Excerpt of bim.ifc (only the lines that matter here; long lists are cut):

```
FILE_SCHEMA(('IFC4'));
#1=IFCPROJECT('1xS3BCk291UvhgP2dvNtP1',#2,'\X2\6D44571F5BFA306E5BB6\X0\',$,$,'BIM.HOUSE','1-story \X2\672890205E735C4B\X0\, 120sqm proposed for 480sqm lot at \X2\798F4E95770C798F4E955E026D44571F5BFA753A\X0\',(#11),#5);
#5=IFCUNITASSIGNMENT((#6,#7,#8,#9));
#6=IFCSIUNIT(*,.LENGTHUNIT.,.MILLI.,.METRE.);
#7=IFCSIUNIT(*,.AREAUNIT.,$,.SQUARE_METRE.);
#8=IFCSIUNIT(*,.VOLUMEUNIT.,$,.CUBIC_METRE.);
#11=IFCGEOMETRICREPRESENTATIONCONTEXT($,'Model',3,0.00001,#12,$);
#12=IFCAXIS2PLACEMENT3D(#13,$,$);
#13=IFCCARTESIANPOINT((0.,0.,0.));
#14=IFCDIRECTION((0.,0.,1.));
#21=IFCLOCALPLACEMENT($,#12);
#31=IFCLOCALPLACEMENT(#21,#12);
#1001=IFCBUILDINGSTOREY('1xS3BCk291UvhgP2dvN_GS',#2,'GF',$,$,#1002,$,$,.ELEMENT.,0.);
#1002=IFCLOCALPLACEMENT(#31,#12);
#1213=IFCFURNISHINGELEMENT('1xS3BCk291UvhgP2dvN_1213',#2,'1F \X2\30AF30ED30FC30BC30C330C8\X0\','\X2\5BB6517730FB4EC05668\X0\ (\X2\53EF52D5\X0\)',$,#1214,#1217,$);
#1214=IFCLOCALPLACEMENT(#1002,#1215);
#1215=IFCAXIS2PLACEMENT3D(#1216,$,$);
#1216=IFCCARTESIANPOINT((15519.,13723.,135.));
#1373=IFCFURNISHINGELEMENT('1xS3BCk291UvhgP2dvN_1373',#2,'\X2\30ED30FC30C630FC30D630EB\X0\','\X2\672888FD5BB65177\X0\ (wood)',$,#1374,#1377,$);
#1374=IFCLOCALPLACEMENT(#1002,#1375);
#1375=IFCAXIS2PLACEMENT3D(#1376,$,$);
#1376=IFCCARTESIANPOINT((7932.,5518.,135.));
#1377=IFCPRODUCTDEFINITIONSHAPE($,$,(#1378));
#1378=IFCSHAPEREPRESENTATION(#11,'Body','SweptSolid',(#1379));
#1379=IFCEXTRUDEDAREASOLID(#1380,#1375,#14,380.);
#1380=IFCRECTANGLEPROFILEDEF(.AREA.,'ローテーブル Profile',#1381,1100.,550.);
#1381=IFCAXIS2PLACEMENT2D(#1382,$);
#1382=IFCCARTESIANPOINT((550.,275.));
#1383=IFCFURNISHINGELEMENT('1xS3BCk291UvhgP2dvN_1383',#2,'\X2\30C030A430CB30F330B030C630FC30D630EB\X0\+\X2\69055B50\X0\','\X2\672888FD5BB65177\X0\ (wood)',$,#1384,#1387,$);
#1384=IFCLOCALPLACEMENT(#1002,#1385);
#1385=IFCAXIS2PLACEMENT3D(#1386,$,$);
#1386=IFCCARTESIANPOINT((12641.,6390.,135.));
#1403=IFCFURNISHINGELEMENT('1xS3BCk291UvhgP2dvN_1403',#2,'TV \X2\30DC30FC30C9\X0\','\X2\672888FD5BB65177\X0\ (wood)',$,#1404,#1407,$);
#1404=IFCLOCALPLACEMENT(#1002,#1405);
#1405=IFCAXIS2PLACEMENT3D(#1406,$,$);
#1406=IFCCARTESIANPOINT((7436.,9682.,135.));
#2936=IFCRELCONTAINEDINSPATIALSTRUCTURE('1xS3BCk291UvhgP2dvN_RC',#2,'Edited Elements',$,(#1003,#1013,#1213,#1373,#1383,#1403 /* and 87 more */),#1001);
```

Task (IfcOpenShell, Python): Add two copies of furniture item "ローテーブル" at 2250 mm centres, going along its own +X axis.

```python
import ifcopenshell
import ifcopenshell.api.geometry
import ifcopenshell.api.root
import ifcopenshell.util.element
import ifcopenshell.util.placement

model = ifcopenshell.open("bim.ifc")


def reuse_history(source, copy):
    """copy_class also copies each property set's owner history, people and application; keep the originals."""
    for rel in copy.IsDefinedBy:
        if rel.is_a("IfcRelDefinesByProperties") and (history := rel.RelatingPropertyDefinition.OwnerHistory):
            rel.RelatingPropertyDefinition.OwnerHistory = source.OwnerHistory
            ifcopenshell.util.element.remove_deep2(model, history)


source = model.by_id(1373)
base = ifcopenshell.util.placement.get_local_placement(source.ObjectPlacement)
step = base[:3, 0] * 2250.0

for i in range(1, 3):
    copy = ifcopenshell.api.root.copy_class(model, product=source)
    copy.Representation = ifcopenshell.util.element.copy_deep(
        model, source.Representation, exclude=["IfcGeometricRepresentationContext", "IfcRepresentationMap"]
    )
    reuse_history(source, copy)
    matrix = base.copy()
    matrix[:3, 3] += i * step
    print("added at", matrix[:3, 3].round(3) + 0.0)
    ifcopenshell.api.geometry.edit_object_placement(model, product=copy, matrix=matrix, is_si=False)

model.write("bim_edited.ifc")
```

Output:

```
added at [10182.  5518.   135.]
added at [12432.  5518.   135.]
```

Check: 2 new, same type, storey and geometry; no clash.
